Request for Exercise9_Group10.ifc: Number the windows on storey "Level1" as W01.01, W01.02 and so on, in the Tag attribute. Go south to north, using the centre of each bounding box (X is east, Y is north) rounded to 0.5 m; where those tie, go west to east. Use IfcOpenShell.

First a look at what the model holds.

```python
import ifcopenshell
import ifcopenshell.util.element
import ifcopenshell.util.placement

model = ifcopenshell.open("Exercise9_Group10.ifc")
print(model.schema)
storey = next(s for s in model.by_type("IfcBuildingStorey") if s.Name == "Level1")
windows = [e for e in ifcopenshell.util.element.get_decomposition(storey) if e.is_a("IfcWindow")]
for e in sorted(windows, key=lambda e: e.id()):
    origin = ifcopenshell.util.placement.get_local_placement(e.ObjectPlacement)[:3, 3]
    print(e.id(), e.Tag, e.Name, origin.round(2) + 0.0, sep=" | ")
```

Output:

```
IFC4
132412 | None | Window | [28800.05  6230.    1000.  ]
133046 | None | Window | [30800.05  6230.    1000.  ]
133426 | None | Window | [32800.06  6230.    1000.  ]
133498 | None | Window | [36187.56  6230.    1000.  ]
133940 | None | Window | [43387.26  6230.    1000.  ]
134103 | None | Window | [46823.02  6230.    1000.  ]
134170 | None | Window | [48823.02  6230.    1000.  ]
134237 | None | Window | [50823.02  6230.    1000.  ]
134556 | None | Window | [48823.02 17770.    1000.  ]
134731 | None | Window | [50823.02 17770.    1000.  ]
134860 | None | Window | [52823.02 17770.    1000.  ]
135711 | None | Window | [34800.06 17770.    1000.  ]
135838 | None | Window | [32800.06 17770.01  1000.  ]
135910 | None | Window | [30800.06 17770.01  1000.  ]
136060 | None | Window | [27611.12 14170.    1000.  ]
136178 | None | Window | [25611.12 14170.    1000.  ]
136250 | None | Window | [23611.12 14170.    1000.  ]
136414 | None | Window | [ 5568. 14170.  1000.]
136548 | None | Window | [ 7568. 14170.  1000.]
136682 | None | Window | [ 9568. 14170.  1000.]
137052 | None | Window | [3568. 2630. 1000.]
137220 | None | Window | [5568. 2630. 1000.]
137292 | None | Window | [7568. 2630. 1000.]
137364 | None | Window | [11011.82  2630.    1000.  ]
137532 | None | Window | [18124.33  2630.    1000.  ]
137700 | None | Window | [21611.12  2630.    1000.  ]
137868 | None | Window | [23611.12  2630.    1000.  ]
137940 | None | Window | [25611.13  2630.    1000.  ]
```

```python
import ifcopenshell
import ifcopenshell.geom
import ifcopenshell.util.element
import ifcopenshell.util.shape

model = ifcopenshell.open("Exercise9_Group10.ifc")
settings = ifcopenshell.geom.settings()
settings.set("use-world-coords", True)


def centre(element):
    shape = ifcopenshell.geom.create_shape(settings, element)
    return ifcopenshell.util.shape.get_bbox_centroid(shape.geometry)


storey = next(s for s in model.by_type("IfcBuildingStorey") if s.Name == "Level1")
windows = [e for e in ifcopenshell.util.element.get_decomposition(storey) if e.is_a("IfcWindow")]

# Insertion points can sit at a corner or the storey origin, so sort by the geometry (in metres).
centres = {e: centre(e) for e in windows}
windows.sort(key=lambda e: (round(centres[e][1] / 0.5), centres[e][0]))

for i, e in enumerate(windows, start=1):
    number = f"W01.{i:02d}"
    e.Tag = number
    print(e.id(), number)

model.write("Exercise9_Group10_v2.ifc")
```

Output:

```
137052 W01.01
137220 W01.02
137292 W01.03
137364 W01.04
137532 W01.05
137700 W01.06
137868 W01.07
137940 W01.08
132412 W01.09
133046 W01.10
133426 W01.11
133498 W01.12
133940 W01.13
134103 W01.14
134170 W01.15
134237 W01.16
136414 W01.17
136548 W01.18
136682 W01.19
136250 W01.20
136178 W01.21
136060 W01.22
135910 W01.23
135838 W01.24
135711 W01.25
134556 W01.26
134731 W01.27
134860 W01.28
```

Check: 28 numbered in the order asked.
